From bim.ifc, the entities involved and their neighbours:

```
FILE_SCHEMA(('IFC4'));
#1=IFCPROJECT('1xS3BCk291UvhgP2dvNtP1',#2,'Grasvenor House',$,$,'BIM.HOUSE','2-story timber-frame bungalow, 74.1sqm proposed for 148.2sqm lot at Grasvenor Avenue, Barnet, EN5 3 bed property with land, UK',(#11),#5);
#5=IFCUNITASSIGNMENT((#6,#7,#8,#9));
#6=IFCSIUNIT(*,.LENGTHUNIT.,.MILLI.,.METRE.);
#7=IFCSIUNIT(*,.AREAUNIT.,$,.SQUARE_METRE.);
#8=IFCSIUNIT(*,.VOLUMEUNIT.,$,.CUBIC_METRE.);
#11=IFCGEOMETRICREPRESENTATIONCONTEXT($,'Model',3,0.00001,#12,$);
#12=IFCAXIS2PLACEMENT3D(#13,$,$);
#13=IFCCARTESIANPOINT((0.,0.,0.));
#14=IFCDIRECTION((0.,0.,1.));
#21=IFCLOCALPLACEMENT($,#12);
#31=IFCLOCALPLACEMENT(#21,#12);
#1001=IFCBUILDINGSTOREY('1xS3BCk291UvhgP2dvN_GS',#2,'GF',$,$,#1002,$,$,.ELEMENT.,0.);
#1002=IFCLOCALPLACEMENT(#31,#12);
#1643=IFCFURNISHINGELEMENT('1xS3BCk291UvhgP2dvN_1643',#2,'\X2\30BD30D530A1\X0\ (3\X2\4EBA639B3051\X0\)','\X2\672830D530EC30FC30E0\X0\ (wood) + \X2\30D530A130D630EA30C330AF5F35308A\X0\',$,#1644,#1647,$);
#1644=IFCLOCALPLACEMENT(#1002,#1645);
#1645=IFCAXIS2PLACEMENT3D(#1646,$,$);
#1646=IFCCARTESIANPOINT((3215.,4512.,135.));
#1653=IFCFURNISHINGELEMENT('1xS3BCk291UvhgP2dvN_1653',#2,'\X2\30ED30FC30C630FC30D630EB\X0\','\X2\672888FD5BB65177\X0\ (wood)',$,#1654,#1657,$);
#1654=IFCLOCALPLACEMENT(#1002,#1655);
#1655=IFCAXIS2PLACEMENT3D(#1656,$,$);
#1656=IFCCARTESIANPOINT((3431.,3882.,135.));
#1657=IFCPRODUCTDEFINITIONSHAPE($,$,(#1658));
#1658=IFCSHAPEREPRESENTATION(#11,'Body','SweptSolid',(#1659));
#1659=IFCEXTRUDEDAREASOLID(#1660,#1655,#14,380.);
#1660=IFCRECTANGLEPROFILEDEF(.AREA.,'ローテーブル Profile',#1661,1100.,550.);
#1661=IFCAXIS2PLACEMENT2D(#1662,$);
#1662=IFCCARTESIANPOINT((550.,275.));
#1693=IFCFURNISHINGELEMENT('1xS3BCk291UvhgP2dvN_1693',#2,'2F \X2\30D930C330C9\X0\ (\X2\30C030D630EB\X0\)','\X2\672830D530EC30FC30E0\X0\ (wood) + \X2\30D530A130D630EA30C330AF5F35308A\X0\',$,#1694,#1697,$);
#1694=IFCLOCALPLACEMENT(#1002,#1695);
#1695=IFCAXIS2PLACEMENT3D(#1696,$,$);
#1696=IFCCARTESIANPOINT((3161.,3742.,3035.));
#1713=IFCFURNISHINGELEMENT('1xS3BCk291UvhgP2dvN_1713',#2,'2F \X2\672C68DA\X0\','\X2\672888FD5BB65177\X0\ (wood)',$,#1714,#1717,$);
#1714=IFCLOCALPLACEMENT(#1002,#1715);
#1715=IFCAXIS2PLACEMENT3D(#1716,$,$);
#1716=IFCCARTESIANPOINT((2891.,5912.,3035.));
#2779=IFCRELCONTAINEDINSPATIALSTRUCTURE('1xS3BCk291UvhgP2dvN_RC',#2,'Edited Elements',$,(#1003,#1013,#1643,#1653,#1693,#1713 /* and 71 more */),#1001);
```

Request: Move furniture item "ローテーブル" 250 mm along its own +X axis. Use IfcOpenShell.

```python
import ifcopenshell
import ifcopenshell.api.geometry
import ifcopenshell.util.placement

model = ifcopenshell.open("bim.ifc")

item = model.by_guid("1xS3BCk291UvhgP2dvN_1653")
matrix = ifcopenshell.util.placement.get_local_placement(item.ObjectPlacement)
matrix[:3, 3] += matrix[:3, 0] * 250.0
ifcopenshell.api.geometry.edit_object_placement(model, product=item, matrix=matrix, is_si=False)

print(ifcopenshell.util.placement.get_local_placement(item.ObjectPlacement).round(3) + 0.0)

model.write("bim_edited.ifc")
```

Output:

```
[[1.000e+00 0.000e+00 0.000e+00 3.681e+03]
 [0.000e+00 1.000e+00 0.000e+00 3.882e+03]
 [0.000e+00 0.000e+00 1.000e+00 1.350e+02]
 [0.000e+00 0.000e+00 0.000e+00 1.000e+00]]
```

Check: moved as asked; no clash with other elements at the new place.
